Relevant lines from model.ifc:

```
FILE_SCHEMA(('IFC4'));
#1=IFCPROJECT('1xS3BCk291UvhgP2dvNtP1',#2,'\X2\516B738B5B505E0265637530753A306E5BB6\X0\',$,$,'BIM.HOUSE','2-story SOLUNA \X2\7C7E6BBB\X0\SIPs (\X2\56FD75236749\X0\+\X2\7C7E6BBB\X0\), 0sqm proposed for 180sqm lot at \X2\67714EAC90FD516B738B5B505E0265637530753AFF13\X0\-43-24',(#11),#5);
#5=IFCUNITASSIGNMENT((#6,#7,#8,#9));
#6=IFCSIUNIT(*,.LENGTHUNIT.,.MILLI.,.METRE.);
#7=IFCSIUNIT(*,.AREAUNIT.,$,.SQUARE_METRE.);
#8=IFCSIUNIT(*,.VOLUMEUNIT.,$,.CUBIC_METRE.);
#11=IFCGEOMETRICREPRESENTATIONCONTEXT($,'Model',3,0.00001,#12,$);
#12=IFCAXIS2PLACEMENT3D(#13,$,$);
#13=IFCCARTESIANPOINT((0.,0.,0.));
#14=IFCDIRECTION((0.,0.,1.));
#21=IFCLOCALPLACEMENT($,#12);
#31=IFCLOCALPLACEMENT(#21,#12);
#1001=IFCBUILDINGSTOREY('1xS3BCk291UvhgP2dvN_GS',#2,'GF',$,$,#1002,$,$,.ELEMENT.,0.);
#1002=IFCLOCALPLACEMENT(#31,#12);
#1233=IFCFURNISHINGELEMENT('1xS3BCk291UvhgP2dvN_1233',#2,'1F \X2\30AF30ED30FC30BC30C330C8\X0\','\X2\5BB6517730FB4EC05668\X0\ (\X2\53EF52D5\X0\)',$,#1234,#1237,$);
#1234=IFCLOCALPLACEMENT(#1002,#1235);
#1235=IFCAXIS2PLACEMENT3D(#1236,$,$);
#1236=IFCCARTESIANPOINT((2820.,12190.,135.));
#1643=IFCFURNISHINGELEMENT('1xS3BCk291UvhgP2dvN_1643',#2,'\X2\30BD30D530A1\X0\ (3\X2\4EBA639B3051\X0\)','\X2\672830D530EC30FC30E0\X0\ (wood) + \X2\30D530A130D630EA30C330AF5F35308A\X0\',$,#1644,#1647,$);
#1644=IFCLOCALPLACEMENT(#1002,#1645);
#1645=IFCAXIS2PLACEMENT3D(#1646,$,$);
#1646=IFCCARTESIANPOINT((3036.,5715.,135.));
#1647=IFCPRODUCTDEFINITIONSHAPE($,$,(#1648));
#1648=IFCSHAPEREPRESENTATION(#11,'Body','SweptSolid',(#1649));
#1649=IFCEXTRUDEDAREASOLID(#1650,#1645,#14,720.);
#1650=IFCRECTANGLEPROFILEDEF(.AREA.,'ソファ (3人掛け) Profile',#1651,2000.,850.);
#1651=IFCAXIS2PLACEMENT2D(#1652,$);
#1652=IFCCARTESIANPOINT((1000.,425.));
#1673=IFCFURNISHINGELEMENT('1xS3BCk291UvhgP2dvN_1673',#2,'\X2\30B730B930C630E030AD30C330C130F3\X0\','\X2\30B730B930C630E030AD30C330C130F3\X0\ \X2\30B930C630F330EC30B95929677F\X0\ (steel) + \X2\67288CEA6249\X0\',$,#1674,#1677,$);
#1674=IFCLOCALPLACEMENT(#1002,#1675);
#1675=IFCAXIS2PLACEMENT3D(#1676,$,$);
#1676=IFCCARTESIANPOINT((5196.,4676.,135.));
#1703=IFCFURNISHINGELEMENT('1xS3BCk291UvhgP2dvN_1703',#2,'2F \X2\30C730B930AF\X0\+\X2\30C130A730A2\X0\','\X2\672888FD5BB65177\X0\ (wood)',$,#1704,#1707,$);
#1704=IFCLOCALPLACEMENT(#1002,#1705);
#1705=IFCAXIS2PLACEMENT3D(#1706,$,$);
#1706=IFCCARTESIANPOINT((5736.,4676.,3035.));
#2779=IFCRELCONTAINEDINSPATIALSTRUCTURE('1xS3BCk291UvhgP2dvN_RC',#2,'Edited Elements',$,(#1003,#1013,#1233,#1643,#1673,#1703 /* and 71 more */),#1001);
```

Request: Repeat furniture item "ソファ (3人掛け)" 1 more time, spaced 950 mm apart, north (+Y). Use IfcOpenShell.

```python
import numpy as np
import ifcopenshell
import ifcopenshell.api.geometry
import ifcopenshell.api.root
import ifcopenshell.util.element
import ifcopenshell.util.placement

model = ifcopenshell.open("model.ifc")


def reuse_history(source, copy):
    """copy_class also copies each property set's owner history, people and application; keep the originals."""
    for rel in copy.IsDefinedBy:
        if rel.is_a("IfcRelDefinesByProperties") and (history := rel.RelatingPropertyDefinition.OwnerHistory):
            rel.RelatingPropertyDefinition.OwnerHistory = source.OwnerHistory
            ifcopenshell.util.element.remove_deep2(model, history)


source = model.by_guid("1xS3BCk291UvhgP2dvN_1643")
base = ifcopenshell.util.placement.get_local_placement(source.ObjectPlacement)
step = np.array([0.0, 1.0, 0.0]) * 950.0

for i in range(1, 2):
    copy = ifcopenshell.api.root.copy_class(model, product=source)
    copy.Representation = ifcopenshell.util.element.copy_deep(
        model, source.Representation, exclude=["IfcGeometricRepresentationContext", "IfcRepresentationMap"]
    )
    reuse_history(source, copy)
    matrix = base.copy()
    matrix[:3, 3] += i * step
    print("added at", matrix[:3, 3].round(3) + 0.0)
    ifcopenshell.api.geometry.edit_object_placement(model, product=copy, matrix=matrix, is_si=False)

model.write("model-out.ifc")
```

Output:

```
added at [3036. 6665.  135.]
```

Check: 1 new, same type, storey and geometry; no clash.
